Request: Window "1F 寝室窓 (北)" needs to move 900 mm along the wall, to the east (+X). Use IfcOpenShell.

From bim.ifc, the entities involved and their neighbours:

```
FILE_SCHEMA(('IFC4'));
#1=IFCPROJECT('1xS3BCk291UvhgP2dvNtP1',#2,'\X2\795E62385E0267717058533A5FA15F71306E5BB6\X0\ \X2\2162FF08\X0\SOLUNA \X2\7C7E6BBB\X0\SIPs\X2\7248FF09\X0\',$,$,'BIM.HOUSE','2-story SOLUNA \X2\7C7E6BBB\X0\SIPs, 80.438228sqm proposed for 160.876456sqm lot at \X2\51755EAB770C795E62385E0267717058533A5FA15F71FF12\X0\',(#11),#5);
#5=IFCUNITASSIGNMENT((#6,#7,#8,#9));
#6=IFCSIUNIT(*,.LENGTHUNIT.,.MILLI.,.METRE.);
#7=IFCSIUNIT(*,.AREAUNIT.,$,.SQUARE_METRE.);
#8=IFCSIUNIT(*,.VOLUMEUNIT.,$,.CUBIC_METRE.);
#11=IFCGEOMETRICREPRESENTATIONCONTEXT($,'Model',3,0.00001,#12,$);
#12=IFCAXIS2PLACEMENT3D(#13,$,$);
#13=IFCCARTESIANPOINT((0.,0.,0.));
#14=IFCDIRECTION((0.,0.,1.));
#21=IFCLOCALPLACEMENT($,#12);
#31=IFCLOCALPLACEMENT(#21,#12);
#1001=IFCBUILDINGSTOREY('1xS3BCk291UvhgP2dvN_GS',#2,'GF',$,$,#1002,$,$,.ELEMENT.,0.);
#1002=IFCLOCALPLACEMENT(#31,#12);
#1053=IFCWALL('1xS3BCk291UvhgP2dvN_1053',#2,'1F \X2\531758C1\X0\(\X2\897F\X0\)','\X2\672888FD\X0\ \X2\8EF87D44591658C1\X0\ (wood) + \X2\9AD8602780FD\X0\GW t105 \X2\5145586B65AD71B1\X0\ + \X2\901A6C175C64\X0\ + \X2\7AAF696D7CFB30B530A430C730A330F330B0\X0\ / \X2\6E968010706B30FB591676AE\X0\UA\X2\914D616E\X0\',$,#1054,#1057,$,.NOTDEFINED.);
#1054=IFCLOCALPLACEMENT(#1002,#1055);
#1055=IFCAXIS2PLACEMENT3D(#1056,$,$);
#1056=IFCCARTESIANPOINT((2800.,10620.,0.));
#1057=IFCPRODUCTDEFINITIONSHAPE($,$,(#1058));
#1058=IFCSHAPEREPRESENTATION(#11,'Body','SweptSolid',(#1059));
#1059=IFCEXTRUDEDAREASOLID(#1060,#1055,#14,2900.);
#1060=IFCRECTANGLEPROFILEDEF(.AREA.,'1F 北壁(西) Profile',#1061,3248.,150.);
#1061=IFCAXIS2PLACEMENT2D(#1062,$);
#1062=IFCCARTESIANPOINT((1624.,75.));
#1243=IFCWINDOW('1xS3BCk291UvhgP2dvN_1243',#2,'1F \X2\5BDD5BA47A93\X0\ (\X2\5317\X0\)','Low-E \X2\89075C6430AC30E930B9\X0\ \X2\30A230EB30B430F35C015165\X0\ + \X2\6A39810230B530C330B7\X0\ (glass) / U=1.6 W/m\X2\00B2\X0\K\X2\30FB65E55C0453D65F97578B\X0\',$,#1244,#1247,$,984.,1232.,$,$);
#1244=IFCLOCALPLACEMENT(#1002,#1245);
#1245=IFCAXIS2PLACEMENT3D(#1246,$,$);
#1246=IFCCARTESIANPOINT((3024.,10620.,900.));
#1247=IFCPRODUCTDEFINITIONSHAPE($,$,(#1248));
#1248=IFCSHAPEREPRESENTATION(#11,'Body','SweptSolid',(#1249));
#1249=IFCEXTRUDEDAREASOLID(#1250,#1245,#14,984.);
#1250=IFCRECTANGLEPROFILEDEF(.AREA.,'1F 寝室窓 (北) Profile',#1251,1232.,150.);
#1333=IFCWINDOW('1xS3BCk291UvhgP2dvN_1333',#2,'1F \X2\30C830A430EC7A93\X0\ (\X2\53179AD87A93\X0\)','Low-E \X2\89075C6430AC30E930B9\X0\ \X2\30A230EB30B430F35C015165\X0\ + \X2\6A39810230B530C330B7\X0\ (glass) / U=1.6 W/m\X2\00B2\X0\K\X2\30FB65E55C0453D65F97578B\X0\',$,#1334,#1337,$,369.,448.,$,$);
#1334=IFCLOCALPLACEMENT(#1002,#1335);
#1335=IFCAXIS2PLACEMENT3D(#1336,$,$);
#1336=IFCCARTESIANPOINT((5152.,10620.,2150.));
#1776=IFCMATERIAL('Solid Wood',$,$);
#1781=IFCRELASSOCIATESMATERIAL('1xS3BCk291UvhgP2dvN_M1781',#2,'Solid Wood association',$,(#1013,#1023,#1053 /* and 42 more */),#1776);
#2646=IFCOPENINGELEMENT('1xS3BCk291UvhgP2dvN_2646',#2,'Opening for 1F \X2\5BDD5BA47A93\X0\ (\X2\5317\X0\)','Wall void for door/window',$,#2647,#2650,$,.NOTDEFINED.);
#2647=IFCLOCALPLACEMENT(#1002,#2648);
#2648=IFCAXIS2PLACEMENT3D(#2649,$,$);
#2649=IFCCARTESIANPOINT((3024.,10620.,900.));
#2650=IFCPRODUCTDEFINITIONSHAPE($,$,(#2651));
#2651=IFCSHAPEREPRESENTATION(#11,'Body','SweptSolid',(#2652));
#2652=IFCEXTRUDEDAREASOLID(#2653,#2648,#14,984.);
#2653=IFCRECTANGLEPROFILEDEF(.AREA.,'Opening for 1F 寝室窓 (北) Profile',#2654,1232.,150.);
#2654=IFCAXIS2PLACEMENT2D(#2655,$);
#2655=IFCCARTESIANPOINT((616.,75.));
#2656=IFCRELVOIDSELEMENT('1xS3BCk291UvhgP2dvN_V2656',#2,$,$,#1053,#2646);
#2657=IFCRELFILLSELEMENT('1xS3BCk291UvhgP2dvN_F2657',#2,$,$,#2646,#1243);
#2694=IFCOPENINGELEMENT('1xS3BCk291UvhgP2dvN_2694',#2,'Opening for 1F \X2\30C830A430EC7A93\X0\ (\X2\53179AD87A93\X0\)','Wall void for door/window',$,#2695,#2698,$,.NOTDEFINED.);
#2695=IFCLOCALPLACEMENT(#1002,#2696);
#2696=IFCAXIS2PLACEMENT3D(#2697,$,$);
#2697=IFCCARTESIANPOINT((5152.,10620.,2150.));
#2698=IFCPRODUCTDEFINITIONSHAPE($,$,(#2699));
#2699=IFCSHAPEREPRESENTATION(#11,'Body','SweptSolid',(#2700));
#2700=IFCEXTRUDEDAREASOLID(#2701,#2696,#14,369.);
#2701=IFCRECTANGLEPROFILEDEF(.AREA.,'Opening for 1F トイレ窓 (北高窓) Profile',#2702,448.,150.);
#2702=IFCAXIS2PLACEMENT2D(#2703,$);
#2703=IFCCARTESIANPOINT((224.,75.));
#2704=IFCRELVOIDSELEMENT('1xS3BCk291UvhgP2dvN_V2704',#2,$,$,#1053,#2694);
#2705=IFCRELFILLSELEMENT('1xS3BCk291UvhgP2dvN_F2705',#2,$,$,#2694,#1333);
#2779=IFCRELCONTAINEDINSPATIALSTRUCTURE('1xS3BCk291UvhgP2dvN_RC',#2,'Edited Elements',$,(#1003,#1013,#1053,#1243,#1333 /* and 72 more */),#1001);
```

```python
import ifcopenshell
import ifcopenshell.api.geometry
import ifcopenshell.util.placement

model = ifcopenshell.open("bim.ifc")

window = model.by_guid("1xS3BCk291UvhgP2dvN_1243")
opening = window.FillsVoids[0].RelatingOpeningElement
wall = opening.VoidsElements[0].RelatingBuildingElement

wall_matrix = ifcopenshell.util.placement.get_local_placement(wall.ObjectPlacement)
shift = wall_matrix[:3, 0] * 900.0
before = ifcopenshell.util.placement.get_local_placement(window.ObjectPlacement)[:3, 3].copy()

# The window is not placed relative to its opening, so move both.
for product in (opening, window):
    matrix = ifcopenshell.util.placement.get_local_placement(product.ObjectPlacement)
    matrix[:3, 3] += shift
    ifcopenshell.api.geometry.edit_object_placement(model, product=product, matrix=matrix, is_si=False)

after = ifcopenshell.util.placement.get_local_placement(window.ObjectPlacement)[:3, 3]
print("window moved by", (after - before).round(3) + 0.0)

model.write("bim_rev.ifc")
```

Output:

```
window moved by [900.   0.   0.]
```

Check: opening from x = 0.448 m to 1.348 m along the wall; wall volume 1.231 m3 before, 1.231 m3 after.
